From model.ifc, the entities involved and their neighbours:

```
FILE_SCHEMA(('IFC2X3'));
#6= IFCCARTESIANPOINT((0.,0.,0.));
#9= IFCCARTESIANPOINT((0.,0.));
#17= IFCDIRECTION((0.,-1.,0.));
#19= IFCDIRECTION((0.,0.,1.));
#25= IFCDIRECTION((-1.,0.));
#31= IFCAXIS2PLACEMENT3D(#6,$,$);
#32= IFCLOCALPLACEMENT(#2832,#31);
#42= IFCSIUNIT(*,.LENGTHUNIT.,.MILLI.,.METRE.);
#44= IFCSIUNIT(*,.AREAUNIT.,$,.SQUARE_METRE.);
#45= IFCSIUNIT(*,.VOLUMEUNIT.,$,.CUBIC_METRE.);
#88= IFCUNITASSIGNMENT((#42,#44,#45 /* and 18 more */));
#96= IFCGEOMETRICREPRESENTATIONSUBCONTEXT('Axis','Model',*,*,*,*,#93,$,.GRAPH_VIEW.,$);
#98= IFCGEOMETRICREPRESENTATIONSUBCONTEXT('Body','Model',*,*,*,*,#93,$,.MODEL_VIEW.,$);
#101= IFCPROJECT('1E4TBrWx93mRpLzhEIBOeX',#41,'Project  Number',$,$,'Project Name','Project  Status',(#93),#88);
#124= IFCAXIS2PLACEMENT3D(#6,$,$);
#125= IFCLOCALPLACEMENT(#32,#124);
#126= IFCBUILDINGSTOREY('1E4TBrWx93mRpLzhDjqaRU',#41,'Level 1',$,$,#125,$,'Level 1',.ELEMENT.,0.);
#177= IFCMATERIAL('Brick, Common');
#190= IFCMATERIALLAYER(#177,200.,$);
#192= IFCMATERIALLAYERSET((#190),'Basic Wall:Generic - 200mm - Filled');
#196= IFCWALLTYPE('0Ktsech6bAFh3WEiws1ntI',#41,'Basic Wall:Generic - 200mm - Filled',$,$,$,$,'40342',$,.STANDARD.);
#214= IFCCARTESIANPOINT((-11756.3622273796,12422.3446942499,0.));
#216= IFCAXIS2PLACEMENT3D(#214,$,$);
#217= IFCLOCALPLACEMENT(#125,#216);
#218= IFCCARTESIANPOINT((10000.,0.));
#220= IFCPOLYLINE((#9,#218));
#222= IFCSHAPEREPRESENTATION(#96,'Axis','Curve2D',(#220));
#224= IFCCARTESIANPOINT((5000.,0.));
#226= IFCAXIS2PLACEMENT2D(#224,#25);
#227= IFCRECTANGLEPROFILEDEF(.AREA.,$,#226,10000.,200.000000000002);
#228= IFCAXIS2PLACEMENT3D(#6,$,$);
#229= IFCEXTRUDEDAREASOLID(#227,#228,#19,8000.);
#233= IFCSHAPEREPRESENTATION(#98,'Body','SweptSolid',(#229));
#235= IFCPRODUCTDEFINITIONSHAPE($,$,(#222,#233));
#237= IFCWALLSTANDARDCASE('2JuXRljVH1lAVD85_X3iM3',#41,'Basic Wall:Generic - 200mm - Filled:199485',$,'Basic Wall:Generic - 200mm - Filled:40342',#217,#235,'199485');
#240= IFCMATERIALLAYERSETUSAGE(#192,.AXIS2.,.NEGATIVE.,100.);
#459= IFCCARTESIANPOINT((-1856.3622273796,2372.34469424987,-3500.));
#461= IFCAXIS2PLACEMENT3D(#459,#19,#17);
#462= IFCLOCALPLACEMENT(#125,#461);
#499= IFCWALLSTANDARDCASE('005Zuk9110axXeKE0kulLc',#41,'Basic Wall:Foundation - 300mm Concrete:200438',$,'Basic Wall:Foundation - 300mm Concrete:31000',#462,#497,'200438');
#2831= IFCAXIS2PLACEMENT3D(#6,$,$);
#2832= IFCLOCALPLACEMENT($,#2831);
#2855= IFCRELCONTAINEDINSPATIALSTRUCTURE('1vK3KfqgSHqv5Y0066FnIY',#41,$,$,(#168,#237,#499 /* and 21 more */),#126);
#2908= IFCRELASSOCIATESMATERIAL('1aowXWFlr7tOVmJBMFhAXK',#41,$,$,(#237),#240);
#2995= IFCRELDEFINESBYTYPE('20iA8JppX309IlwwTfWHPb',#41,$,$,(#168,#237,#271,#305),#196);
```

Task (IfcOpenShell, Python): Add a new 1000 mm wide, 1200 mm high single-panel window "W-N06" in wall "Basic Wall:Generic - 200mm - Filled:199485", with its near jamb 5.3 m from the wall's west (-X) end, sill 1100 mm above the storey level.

```python
import numpy as np
import ifcopenshell
import ifcopenshell.api.feature
import ifcopenshell.api.geometry
import ifcopenshell.api.root
import ifcopenshell.api.spatial
import ifcopenshell.api.type
import ifcopenshell.geom
import ifcopenshell.util.element
import ifcopenshell.util.placement
import ifcopenshell.util.representation
import ifcopenshell.util.shape
import ifcopenshell.util.unit

model = ifcopenshell.open("model.ifc")
unit_scale = ifcopenshell.util.unit.calculate_unit_scale(model)
settings = ifcopenshell.geom.settings()


def volume(element):
    """Net volume in cubic metres, openings subtracted."""
    shape = ifcopenshell.geom.create_shape(settings, element)
    return ifcopenshell.util.shape.get_volume(shape.geometry)


wall = model.by_guid("2JuXRljVH1lAVD85_X3iM3")
storey = ifcopenshell.util.element.get_container(wall, ifc_class="IfcBuildingStorey")
context = ifcopenshell.util.representation.get_context(model, "Model", "Body", "MODEL_VIEW")
before = volume(wall)

width, height, from_end, sill = 1, 1.2, 5.3, 1.1  # metres

# The wall runs along its own X axis, and the end named is its -X end.
wall_shape = ifcopenshell.geom.create_shape(settings, wall)
x, y, z = ifcopenshell.util.shape.get_vertices(wall_shape.geometry).T
start = x.min() + from_end
face, thickness = float(y.min()), float(y.max() - y.min())
wall_matrix = ifcopenshell.util.placement.get_local_placement(wall.ObjectPlacement)
level = ifcopenshell.util.placement.get_local_placement(storey.ObjectPlacement)[2, 3]


def in_wall(x, y):
    """Placement at x, y metres in the wall's axes, at sill height."""
    matrix = wall_matrix.copy()
    matrix[:, 3] = wall_matrix @ np.array([x / unit_scale, y / unit_scale, 0.0, 1.0])
    matrix[2, 3] = level + sill / unit_scale
    return matrix


# Opening: a box that overshoots both wall faces by 50 mm.
opening = ifcopenshell.api.root.create_entity(model, ifc_class="IfcOpeningElement")
box = ifcopenshell.api.geometry.add_wall_representation(
    model, context=context, length=width, height=height, thickness=thickness + 0.1
)
ifcopenshell.api.geometry.assign_representation(model, product=opening, representation=box)
ifcopenshell.api.geometry.edit_object_placement(model, product=opening, matrix=in_wall(start, face - 0.05), is_si=False)
ifcopenshell.api.feature.add_feature(model, feature=opening, element=wall)

window = ifcopenshell.api.root.create_entity(model, ifc_class="IfcWindow", name="W-N06")
window.OverallWidth, window.OverallHeight = width / unit_scale, height / unit_scale
body = ifcopenshell.api.geometry.add_window_representation(
    model,
    context=context,
    overall_width=window.OverallWidth,
    overall_height=window.OverallHeight,
    partition_type="SINGLE_PANEL",
)
ifcopenshell.api.geometry.assign_representation(model, product=window, representation=body)
ifcopenshell.api.spatial.assign_container(model, products=[window], relating_structure=storey)
fills = ifcopenshell.api.feature.add_filling(model, opening=opening, element=window)
fills.OwnerHistory = window.OwnerHistory  # required in IFC2X3

# IFC2X3 keeps the operation on the window style.
style = ifcopenshell.api.root.create_entity(model, ifc_class="IfcWindowStyle", name="W-N06")
style.OperationType, style.ConstructionType = "SINGLE_PANEL", "NOTDEFINED"
style.ParameterTakesPrecedence = style.Sizeable = False
ifcopenshell.api.type.assign_type(model, related_objects=[window], relating_type=style)

# Centre the window in the wall's thickness.
ifcopenshell.api.geometry.edit_object_placement(model, product=window, matrix=in_wall(start, face), is_si=False)
window_shape = ifcopenshell.geom.create_shape(settings, window)
depth = ifcopenshell.util.shape.get_vertices(window_shape.geometry)[:, 1]
offset = face + thickness / 2 - (depth.min() + depth.max()) / 2
ifcopenshell.api.geometry.edit_object_placement(model, product=window, matrix=in_wall(start, offset), is_si=False)

after = volume(wall)

print(f"wall volume {before:.3f} -> {after:.3f} m3")

model.write("model_v2.ifc")
```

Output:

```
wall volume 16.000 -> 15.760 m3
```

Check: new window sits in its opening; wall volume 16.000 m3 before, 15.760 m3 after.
